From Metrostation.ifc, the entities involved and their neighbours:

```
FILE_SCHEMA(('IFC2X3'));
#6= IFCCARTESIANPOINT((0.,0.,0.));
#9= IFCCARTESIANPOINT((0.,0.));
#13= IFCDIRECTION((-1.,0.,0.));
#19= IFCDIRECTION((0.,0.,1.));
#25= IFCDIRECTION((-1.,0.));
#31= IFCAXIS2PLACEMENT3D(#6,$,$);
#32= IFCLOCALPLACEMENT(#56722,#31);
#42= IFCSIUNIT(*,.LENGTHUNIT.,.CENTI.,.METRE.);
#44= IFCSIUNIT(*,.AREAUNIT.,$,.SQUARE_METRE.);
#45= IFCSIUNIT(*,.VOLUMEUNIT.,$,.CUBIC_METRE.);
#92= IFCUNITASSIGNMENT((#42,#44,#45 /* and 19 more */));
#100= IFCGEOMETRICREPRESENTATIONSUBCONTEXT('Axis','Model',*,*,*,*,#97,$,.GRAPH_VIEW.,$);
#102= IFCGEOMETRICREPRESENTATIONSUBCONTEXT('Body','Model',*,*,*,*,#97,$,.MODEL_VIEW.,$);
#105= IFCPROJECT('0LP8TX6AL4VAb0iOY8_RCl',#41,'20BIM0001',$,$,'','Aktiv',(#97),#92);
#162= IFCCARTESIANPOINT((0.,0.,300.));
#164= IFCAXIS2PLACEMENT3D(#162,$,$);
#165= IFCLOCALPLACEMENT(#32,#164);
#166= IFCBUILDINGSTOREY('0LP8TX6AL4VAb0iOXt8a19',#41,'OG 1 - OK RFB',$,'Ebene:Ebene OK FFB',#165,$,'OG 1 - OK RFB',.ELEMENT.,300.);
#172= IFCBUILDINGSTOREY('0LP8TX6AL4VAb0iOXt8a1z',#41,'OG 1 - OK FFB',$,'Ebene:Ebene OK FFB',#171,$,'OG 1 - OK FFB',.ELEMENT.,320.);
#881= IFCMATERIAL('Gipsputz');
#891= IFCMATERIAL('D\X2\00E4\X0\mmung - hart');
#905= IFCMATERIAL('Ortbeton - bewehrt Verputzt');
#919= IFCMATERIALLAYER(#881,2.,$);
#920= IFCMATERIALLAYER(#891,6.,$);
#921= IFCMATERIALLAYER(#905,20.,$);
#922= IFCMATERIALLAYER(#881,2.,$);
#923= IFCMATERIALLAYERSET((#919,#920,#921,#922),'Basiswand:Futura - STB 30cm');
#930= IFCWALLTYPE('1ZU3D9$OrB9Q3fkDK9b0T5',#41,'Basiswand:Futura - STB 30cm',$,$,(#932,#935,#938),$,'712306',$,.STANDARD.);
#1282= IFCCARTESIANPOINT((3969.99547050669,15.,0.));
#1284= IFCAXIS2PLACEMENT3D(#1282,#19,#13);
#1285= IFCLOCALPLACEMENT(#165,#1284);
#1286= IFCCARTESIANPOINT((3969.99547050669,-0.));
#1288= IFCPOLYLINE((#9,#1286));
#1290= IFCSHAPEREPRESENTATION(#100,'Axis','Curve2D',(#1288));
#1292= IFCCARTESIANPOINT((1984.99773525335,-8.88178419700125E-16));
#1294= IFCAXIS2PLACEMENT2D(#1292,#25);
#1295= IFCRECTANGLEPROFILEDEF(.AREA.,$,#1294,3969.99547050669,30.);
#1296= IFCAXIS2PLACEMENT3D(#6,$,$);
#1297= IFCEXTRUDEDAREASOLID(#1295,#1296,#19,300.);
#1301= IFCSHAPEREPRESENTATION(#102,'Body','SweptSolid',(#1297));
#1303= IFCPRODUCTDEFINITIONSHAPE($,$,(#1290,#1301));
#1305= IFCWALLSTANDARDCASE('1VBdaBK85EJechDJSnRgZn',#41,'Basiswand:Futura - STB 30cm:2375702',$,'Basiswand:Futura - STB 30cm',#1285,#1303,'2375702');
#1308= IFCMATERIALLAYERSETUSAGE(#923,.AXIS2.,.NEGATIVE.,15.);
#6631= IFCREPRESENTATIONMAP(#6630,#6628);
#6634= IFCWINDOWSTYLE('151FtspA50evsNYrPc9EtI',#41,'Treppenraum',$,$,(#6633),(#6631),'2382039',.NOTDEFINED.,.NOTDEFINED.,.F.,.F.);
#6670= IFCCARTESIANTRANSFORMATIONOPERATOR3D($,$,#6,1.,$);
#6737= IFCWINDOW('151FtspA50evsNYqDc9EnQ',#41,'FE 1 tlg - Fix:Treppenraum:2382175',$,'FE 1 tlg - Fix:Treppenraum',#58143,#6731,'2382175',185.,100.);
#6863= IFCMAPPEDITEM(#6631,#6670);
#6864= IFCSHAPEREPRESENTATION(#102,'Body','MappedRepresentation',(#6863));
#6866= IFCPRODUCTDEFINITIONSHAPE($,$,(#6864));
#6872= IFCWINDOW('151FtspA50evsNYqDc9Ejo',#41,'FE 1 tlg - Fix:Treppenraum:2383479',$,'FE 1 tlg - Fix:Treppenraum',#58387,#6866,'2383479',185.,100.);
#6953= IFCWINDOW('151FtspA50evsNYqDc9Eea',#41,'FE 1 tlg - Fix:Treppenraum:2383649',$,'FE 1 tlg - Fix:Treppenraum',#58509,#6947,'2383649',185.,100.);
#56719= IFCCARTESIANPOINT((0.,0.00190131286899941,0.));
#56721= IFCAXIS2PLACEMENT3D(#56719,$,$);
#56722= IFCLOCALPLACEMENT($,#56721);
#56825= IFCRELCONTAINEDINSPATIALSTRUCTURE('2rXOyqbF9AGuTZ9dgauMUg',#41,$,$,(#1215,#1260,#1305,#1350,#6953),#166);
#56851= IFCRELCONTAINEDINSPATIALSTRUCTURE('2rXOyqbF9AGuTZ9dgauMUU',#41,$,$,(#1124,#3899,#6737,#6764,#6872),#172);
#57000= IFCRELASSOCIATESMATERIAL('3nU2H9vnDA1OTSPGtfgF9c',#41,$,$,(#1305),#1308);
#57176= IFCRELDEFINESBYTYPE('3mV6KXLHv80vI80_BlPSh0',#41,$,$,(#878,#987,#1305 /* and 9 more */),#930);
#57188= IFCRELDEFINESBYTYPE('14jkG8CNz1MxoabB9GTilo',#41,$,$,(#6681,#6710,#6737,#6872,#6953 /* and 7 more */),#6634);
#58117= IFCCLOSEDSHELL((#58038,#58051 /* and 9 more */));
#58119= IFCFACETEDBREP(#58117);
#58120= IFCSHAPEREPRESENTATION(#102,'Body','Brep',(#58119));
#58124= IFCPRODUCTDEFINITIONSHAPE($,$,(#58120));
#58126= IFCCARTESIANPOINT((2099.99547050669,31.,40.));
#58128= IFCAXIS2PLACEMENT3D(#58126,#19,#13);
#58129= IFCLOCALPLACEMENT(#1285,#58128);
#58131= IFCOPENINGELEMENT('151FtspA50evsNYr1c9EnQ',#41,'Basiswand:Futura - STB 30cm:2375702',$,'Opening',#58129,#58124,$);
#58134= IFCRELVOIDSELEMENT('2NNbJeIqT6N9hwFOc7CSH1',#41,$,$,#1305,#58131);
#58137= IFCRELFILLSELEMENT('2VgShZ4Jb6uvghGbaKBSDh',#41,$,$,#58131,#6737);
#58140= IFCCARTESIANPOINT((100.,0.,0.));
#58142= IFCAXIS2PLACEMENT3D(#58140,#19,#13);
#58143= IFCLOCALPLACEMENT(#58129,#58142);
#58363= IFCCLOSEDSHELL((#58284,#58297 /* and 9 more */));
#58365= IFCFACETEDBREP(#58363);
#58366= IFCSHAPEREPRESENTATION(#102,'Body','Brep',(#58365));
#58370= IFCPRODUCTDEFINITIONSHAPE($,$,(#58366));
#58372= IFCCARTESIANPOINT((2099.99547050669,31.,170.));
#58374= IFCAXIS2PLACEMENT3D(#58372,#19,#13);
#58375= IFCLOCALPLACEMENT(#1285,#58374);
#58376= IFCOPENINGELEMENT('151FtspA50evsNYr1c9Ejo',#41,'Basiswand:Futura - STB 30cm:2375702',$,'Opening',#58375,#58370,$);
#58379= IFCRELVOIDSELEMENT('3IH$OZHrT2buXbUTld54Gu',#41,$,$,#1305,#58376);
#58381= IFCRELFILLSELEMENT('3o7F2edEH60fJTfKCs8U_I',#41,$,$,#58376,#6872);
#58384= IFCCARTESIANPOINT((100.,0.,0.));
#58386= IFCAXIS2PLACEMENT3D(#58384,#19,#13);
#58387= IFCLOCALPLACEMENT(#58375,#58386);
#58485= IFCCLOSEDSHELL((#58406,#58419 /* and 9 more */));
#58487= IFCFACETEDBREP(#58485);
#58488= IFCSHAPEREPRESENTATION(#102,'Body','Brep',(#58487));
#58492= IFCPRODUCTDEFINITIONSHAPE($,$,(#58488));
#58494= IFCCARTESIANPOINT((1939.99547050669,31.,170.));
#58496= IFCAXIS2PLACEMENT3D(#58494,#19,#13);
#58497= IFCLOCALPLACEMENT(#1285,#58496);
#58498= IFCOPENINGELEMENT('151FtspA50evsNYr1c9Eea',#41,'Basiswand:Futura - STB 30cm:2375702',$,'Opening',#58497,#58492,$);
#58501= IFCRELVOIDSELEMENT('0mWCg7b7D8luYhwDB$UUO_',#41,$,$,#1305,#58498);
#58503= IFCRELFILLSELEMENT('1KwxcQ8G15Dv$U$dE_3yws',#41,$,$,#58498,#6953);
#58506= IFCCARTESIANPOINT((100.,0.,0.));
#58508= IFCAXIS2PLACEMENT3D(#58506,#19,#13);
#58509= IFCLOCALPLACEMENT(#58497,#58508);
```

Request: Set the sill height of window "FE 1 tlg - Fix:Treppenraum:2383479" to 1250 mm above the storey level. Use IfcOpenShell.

```python
import numpy as np
import ifcopenshell
import ifcopenshell.api.geometry
import ifcopenshell.geom
import ifcopenshell.util.element
import ifcopenshell.util.placement
import ifcopenshell.util.shape
import ifcopenshell.util.unit

model = ifcopenshell.open("Metrostation.ifc")
unit_scale = ifcopenshell.util.unit.calculate_unit_scale(model)

window = model.by_guid("151FtspA50evsNYqDc9Ejo")
opening = window.FillsVoids[0].RelatingOpeningElement
storey = ifcopenshell.util.element.get_container(window, ifc_class="IfcBuildingStorey")
level = ifcopenshell.util.placement.get_local_placement(storey.ObjectPlacement)[2, 3]

# The opening's origin need not be at the sill, so measure its lowest point.
shape = ifcopenshell.geom.create_shape(ifcopenshell.geom.settings(), opening)
bottom = ifcopenshell.util.shape.get_shape_bottom_elevation(shape, shape.geometry) / unit_scale
dz = level + 1.25 / unit_scale - bottom

shift = np.array([0.0, 0.0, dz])
# The window is placed relative to its opening, so it follows when the opening moves.
matrix = ifcopenshell.util.placement.get_local_placement(opening.ObjectPlacement)
matrix[:3, 3] += shift
ifcopenshell.api.geometry.edit_object_placement(
    model, product=opening, matrix=matrix, is_si=False, should_transform_children=True
)

print(f"moved by {dz * unit_scale:+.3f} m")

model.write("Metrostation_updated.ifc")
```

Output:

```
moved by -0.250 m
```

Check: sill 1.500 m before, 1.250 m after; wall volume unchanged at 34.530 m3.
